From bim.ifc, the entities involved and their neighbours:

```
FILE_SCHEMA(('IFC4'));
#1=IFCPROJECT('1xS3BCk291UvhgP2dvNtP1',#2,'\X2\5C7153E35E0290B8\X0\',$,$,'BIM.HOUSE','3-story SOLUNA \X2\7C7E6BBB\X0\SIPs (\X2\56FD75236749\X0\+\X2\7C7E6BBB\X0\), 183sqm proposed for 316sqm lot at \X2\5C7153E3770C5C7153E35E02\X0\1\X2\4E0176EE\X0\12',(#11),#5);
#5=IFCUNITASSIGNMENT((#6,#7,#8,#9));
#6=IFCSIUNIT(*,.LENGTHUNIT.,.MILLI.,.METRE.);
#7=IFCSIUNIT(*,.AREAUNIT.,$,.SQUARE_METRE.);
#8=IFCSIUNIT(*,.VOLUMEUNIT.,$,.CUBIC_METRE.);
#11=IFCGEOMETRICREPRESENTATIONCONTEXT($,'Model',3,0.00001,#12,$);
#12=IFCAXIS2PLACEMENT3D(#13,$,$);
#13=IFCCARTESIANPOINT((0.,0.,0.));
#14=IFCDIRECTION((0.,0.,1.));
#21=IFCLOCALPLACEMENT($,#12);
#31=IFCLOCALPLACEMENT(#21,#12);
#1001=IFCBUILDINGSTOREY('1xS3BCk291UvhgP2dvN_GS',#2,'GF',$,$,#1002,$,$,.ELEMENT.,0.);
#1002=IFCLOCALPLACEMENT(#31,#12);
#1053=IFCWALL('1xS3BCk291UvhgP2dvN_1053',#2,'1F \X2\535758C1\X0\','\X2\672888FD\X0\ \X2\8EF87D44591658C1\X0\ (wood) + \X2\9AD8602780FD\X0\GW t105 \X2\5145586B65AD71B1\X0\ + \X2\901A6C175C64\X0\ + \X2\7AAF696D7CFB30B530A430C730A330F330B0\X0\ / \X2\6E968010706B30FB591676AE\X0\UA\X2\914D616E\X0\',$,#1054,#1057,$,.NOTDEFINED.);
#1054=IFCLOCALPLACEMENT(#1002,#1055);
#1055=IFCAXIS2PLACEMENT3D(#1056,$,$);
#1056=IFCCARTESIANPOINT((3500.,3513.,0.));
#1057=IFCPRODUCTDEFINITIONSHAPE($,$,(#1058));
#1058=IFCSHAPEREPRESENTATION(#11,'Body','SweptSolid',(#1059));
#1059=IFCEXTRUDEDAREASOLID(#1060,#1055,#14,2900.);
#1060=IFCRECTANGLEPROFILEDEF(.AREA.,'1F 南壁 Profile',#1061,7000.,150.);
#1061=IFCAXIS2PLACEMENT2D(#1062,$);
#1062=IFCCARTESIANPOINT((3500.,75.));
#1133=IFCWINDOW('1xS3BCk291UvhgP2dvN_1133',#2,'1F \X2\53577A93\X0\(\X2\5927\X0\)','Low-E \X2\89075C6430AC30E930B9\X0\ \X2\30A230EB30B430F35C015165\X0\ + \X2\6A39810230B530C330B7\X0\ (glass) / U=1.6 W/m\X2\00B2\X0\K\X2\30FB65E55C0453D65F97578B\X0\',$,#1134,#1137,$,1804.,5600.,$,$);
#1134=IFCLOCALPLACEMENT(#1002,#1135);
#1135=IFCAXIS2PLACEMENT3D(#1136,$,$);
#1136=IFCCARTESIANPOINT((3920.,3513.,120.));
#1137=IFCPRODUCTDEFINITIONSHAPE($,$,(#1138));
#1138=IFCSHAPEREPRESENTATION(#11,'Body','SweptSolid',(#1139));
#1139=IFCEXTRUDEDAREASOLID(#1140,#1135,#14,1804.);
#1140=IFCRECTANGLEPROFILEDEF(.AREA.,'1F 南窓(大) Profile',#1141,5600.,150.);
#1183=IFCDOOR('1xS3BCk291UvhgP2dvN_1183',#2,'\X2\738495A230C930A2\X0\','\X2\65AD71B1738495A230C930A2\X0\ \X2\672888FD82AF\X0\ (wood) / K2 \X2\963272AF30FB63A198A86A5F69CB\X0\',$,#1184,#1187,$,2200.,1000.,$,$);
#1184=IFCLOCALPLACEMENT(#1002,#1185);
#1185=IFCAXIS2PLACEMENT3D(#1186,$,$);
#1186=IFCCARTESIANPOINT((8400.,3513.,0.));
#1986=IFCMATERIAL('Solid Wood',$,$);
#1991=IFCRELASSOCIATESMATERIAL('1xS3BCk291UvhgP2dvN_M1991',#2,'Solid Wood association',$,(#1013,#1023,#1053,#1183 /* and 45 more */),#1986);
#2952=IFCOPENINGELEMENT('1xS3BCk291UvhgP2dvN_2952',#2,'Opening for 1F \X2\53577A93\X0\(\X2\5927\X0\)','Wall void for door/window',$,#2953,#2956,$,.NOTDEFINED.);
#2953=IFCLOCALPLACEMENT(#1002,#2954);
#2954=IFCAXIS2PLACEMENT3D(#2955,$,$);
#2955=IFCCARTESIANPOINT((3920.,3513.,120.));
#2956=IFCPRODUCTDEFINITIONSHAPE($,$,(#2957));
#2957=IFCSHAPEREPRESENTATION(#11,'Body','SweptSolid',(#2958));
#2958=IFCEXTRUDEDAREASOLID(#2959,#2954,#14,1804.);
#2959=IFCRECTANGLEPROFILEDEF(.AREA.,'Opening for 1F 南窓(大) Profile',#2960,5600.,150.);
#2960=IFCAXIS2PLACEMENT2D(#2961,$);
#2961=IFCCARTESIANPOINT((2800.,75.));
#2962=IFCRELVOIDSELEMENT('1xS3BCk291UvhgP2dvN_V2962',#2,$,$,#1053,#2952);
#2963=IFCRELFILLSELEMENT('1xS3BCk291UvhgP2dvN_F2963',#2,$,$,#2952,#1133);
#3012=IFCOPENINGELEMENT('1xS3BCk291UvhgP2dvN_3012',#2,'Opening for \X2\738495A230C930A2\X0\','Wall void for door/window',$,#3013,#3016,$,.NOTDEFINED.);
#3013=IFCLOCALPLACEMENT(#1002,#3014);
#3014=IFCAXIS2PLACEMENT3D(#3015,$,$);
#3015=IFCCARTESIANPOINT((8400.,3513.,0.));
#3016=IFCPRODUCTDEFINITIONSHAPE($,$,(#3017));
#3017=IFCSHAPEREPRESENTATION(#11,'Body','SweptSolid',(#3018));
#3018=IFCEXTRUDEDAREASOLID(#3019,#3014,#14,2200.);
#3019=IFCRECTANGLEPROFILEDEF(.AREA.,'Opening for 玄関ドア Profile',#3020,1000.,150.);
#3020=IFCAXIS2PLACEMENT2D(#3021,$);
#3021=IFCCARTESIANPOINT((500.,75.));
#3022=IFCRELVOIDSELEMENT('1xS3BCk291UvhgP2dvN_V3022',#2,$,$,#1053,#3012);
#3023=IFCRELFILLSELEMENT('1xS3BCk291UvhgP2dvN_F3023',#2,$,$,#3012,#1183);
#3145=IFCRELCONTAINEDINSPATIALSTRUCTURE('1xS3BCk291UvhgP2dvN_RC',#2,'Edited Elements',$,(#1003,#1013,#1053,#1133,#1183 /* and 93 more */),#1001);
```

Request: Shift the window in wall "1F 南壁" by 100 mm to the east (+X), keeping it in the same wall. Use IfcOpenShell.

```python
import ifcopenshell
import ifcopenshell.api.geometry
import ifcopenshell.util.placement
import ifcopenshell.util.unit

model = ifcopenshell.open("bim.ifc")
unit_scale = ifcopenshell.util.unit.calculate_unit_scale(model)

window = model.by_id(1133)
opening = window.FillsVoids[0].RelatingOpeningElement
wall = opening.VoidsElements[0].RelatingBuildingElement

wall_matrix = ifcopenshell.util.placement.get_local_placement(wall.ObjectPlacement)
shift = wall_matrix[:3, 0] * 0.1 / unit_scale
before = ifcopenshell.util.placement.get_local_placement(window.ObjectPlacement)[:3, 3].copy()

# The window is not placed relative to its opening, so move both.
for product in (opening, window):
    matrix = ifcopenshell.util.placement.get_local_placement(product.ObjectPlacement)
    matrix[:3, 3] += shift
    ifcopenshell.api.geometry.edit_object_placement(model, product=product, matrix=matrix, is_si=False)

after = ifcopenshell.util.placement.get_local_placement(window.ObjectPlacement)[:3, 3]
print("window moved by", (after - before).round(3) + 0.0)

model.write("bim_v2.ifc")
```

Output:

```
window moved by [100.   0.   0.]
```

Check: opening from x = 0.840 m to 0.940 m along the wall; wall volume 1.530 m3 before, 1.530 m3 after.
